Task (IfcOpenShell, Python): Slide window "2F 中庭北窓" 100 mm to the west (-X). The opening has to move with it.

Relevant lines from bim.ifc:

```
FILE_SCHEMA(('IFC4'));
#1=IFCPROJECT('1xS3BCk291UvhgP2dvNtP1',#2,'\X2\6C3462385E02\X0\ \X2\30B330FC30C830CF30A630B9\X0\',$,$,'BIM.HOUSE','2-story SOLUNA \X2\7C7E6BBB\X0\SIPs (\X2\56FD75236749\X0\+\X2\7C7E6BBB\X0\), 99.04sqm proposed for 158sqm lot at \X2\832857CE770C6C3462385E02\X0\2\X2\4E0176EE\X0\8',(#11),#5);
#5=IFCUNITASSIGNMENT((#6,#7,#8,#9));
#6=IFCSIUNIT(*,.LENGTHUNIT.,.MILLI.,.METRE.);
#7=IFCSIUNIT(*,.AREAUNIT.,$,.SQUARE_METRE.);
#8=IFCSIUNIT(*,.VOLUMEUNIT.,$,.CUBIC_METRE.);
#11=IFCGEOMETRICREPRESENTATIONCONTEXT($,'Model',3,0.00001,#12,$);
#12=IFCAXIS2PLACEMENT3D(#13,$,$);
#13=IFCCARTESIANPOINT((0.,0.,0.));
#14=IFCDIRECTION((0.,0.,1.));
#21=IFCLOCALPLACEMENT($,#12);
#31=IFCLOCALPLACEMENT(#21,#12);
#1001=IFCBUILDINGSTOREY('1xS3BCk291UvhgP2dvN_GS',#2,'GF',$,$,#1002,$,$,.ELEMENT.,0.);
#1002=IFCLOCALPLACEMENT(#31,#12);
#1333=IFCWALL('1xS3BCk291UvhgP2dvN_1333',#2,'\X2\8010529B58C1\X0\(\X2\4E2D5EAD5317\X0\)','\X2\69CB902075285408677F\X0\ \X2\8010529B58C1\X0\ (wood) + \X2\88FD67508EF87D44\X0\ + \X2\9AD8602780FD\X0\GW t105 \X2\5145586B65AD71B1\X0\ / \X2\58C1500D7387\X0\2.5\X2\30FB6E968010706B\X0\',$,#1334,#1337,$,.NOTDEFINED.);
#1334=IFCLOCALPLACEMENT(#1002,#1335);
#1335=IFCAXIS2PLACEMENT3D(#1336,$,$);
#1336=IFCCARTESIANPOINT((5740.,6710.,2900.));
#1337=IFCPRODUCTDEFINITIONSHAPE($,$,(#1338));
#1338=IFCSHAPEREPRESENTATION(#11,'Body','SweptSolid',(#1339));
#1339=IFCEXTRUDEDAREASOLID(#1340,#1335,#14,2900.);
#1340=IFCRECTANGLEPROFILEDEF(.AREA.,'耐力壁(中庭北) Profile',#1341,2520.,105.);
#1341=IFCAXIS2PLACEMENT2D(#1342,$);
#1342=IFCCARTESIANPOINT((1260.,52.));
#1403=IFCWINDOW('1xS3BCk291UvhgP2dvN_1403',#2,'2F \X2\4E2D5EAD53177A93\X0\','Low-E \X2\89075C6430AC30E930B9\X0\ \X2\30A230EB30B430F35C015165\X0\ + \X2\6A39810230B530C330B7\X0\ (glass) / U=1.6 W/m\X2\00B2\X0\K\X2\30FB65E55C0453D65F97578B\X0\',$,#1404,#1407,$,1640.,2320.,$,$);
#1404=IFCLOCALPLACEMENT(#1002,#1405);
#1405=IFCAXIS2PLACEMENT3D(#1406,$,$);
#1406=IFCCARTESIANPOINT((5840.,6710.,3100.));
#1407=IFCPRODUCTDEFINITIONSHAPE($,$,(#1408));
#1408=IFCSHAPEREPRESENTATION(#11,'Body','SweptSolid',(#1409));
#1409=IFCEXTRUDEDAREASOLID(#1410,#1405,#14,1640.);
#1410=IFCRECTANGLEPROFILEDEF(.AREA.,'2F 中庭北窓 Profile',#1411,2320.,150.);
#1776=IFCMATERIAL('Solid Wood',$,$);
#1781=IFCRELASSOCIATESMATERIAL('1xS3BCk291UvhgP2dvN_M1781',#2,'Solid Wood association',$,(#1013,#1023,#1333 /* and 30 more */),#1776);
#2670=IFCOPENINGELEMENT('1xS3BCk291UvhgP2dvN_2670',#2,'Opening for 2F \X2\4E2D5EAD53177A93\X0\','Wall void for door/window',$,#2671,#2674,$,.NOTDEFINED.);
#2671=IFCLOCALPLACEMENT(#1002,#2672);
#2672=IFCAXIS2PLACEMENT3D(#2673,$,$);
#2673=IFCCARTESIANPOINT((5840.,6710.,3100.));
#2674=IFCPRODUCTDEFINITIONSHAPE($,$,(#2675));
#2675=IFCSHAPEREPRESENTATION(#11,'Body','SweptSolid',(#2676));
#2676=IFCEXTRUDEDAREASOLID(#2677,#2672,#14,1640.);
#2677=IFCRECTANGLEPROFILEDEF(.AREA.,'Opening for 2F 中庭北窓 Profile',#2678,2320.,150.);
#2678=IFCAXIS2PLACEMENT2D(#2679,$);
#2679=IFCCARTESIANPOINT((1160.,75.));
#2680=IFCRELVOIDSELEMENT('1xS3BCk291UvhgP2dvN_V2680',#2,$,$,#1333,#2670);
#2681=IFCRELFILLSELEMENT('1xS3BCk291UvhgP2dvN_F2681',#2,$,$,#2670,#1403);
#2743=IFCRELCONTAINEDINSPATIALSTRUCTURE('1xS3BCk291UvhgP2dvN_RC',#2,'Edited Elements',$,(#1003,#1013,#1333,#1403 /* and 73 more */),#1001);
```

```python
import ifcopenshell
import ifcopenshell.api.geometry
import ifcopenshell.util.placement
import ifcopenshell.util.unit

model = ifcopenshell.open("bim.ifc")
unit_scale = ifcopenshell.util.unit.calculate_unit_scale(model)

window = model.by_id(1403)
opening = window.FillsVoids[0].RelatingOpeningElement
wall = opening.VoidsElements[0].RelatingBuildingElement

wall_matrix = ifcopenshell.util.placement.get_local_placement(wall.ObjectPlacement)
shift = wall_matrix[:3, 0] * -0.1 / unit_scale
before = ifcopenshell.util.placement.get_local_placement(window.ObjectPlacement)[:3, 3].copy()

# The window is not placed relative to its opening, so move both.
for product in (opening, window):
    matrix = ifcopenshell.util.placement.get_local_placement(product.ObjectPlacement)
    matrix[:3, 3] += shift
    ifcopenshell.api.geometry.edit_object_placement(model, product=product, matrix=matrix, is_si=False)

after = ifcopenshell.util.placement.get_local_placement(window.ObjectPlacement)[:3, 3]
print("window moved by", (after - before).round(3) + 0.0)

model.write("bim_rev.ifc")
```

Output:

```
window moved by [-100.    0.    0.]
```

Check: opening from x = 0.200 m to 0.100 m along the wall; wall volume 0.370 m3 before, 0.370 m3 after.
